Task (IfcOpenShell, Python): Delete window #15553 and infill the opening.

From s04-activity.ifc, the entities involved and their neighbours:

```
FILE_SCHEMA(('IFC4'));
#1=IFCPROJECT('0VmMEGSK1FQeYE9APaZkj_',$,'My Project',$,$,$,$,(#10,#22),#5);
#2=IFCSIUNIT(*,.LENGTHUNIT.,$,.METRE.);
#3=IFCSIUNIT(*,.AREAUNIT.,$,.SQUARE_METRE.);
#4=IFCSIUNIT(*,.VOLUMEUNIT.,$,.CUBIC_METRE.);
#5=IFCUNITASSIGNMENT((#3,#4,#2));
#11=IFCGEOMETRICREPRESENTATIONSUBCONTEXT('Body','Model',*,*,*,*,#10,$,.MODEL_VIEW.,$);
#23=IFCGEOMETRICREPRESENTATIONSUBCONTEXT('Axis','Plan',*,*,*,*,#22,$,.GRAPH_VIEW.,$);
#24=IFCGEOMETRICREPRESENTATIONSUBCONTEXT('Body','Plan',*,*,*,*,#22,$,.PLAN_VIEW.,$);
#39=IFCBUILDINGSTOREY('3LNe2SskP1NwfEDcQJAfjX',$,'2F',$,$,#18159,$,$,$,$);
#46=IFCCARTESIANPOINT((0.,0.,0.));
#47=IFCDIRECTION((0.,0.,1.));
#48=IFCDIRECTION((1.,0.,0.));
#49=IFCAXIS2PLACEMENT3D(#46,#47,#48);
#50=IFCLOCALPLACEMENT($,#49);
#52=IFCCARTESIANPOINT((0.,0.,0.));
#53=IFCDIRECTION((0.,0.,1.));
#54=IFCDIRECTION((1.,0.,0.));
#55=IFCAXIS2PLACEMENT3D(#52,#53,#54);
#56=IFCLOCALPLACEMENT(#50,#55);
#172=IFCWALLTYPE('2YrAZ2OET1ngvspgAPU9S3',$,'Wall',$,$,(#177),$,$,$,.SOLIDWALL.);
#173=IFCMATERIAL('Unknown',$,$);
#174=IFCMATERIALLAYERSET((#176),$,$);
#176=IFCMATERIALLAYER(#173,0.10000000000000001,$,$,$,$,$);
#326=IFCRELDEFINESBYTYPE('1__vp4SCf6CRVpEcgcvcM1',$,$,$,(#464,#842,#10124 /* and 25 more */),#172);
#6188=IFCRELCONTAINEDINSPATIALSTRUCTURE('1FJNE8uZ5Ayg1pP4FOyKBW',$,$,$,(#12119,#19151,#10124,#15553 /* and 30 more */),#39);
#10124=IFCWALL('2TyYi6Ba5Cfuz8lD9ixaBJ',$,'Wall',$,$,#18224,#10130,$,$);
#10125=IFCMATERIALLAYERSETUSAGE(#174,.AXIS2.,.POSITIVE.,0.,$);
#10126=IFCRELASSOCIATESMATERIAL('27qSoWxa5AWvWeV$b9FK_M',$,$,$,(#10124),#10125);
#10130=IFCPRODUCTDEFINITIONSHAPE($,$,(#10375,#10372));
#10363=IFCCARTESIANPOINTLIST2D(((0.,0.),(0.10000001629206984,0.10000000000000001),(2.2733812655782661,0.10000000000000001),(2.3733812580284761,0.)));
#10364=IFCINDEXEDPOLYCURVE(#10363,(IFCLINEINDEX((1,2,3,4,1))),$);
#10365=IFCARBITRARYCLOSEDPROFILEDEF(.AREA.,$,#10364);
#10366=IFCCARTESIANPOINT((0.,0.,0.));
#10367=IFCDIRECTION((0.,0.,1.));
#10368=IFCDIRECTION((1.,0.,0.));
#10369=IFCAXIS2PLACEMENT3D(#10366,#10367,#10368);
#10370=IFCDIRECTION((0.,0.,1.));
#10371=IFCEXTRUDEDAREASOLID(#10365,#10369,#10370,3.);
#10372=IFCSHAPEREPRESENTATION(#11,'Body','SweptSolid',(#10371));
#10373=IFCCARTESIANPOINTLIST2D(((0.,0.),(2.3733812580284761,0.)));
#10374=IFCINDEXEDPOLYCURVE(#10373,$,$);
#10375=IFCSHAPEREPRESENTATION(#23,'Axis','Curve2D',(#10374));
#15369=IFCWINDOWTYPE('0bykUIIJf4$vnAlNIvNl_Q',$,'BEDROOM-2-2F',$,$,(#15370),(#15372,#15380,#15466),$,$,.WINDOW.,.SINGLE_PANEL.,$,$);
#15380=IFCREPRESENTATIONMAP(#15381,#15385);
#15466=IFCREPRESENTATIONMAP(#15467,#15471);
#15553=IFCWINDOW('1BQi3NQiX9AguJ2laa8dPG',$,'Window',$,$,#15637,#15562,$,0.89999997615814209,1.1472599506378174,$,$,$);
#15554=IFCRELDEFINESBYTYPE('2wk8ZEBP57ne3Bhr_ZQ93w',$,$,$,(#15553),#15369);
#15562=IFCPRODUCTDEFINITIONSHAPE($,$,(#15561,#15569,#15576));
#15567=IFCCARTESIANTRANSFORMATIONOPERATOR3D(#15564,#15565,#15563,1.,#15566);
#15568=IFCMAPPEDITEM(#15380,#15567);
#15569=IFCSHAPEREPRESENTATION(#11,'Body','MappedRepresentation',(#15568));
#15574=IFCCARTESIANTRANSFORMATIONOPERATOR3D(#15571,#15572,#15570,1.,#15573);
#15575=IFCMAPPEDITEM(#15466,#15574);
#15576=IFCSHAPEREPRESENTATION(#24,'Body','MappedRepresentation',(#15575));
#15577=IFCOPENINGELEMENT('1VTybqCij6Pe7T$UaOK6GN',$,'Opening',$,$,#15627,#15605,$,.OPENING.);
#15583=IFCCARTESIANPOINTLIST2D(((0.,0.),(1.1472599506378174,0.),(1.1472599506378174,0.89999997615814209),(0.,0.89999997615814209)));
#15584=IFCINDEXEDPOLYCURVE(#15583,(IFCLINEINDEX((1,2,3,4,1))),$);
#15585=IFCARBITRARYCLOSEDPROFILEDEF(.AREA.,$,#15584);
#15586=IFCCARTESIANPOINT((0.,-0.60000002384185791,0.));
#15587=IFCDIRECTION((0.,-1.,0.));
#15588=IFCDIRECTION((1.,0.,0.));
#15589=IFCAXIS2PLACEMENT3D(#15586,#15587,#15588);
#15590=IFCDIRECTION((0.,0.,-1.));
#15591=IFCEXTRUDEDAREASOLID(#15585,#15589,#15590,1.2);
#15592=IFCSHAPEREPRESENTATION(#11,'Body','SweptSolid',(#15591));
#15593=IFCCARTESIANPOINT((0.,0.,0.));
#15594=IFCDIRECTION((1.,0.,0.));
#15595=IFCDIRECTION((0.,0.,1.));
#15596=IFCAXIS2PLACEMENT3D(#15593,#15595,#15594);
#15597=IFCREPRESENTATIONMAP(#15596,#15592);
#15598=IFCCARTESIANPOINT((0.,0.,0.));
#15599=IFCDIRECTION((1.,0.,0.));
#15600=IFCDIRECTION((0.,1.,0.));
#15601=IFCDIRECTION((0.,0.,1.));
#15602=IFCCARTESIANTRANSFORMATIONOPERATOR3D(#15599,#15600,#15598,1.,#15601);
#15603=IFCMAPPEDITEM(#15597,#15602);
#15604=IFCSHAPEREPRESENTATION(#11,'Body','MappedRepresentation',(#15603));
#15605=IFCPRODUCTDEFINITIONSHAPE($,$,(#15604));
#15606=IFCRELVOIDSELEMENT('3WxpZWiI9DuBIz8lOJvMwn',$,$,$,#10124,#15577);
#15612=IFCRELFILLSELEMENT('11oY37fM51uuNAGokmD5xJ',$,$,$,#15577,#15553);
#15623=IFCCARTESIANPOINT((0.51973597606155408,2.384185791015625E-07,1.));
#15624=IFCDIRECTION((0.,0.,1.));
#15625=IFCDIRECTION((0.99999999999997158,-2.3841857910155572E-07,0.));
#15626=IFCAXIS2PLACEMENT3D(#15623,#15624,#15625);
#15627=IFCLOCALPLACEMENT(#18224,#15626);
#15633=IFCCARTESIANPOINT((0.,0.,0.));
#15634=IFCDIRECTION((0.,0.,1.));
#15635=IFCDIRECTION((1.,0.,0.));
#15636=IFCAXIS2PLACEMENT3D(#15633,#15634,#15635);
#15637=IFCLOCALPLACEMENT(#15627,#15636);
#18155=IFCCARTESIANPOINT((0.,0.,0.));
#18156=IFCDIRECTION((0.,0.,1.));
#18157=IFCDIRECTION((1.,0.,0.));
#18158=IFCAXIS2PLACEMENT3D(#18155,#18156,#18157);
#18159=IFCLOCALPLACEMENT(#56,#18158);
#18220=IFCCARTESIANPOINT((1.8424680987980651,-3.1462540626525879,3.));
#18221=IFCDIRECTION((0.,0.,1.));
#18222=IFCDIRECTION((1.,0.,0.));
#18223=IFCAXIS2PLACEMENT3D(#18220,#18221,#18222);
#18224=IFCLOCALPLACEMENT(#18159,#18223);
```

```python
import ifcopenshell
import ifcopenshell.api.feature
import ifcopenshell.api.root
import ifcopenshell.geom
import ifcopenshell.util.shape

model = ifcopenshell.open("s04-activity.ifc")
settings = ifcopenshell.geom.settings()


def volume(element):
    """Net volume in cubic metres, openings subtracted."""
    shape = ifcopenshell.geom.create_shape(settings, element)
    return ifcopenshell.util.shape.get_volume(shape.geometry)


window = model.by_id(15553)
opening = window.FillsVoids[0].RelatingOpeningElement
wall = opening.VoidsElements[0].RelatingBuildingElement
before = volume(wall)

ifcopenshell.api.root.remove_product(model, product=window)
ifcopenshell.api.feature.remove_feature(model, feature=opening)

after = volume(wall)

print(f"wall volume {before:.3f} -> {after:.3f} m3")

model.write("s04-activity_edited.ifc")
```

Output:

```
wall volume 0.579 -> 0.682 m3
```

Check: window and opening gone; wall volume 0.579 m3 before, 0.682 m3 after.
